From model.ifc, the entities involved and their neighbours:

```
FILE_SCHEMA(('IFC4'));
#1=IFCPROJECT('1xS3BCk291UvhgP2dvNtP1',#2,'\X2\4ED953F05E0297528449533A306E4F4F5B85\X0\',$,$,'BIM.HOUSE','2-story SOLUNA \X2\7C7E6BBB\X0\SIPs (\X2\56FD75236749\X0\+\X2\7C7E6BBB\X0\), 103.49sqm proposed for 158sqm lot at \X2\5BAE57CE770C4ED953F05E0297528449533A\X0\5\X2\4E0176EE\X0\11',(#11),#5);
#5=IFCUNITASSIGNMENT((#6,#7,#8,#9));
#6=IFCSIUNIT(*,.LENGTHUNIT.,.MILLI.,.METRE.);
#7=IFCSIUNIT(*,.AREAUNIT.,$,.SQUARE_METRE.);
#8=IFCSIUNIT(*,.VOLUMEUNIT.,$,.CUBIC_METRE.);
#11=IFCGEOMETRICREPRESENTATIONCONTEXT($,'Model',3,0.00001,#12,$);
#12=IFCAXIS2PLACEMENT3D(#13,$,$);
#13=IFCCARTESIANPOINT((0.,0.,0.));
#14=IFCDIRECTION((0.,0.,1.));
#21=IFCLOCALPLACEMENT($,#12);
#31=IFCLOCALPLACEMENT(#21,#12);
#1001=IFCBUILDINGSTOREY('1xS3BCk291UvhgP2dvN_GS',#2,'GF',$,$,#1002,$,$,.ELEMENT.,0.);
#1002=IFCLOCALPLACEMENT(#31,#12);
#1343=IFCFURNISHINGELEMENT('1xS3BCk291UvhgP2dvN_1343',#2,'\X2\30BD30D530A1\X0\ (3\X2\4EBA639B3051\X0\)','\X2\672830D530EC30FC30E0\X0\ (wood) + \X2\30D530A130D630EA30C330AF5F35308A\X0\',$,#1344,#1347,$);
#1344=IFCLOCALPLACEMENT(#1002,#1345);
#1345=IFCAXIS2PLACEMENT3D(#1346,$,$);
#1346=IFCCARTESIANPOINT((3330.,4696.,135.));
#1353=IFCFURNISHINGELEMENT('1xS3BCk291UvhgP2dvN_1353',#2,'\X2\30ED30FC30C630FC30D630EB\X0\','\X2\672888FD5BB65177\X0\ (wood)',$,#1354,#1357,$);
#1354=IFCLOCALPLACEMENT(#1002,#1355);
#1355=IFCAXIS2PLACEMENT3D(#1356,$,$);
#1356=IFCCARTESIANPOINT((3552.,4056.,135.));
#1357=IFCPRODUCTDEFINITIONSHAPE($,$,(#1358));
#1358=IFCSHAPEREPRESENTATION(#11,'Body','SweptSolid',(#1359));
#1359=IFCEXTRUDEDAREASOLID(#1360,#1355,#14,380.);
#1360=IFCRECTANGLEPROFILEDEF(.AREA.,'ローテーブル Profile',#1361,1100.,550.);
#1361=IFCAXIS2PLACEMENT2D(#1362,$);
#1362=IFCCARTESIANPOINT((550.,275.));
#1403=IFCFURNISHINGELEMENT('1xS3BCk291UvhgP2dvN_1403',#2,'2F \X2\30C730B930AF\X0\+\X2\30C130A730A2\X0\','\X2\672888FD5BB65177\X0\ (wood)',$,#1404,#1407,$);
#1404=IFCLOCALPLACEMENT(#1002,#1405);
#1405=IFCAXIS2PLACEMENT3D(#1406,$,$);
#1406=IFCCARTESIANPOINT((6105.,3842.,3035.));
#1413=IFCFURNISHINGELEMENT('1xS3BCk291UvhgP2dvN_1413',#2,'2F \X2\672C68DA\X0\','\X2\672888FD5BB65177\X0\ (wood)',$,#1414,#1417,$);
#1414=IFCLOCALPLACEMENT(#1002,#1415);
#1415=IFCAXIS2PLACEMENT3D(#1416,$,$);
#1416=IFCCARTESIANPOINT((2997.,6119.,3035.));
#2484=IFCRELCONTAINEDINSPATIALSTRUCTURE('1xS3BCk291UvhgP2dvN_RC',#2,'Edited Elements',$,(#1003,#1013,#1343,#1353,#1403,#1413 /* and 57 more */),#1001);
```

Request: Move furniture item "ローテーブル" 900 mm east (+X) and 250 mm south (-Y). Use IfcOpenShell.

```python
import ifcopenshell
import ifcopenshell.api.geometry
import ifcopenshell.util.placement
import ifcopenshell.util.unit

model = ifcopenshell.open("model.ifc")
unit_scale = ifcopenshell.util.unit.calculate_unit_scale(model)

item = model.by_id(1353)
matrix = ifcopenshell.util.placement.get_local_placement(item.ObjectPlacement)
matrix[0, 3] += 0.9 / unit_scale
matrix[1, 3] -= 0.25 / unit_scale
ifcopenshell.api.geometry.edit_object_placement(model, product=item, matrix=matrix, is_si=False)

print(ifcopenshell.util.placement.get_local_placement(item.ObjectPlacement).round(3) + 0.0)

model.write("model_rev.ifc")
```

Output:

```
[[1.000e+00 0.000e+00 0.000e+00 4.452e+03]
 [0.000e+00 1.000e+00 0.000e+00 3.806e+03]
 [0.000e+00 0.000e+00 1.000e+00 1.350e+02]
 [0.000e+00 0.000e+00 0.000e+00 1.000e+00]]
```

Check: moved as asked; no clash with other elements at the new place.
